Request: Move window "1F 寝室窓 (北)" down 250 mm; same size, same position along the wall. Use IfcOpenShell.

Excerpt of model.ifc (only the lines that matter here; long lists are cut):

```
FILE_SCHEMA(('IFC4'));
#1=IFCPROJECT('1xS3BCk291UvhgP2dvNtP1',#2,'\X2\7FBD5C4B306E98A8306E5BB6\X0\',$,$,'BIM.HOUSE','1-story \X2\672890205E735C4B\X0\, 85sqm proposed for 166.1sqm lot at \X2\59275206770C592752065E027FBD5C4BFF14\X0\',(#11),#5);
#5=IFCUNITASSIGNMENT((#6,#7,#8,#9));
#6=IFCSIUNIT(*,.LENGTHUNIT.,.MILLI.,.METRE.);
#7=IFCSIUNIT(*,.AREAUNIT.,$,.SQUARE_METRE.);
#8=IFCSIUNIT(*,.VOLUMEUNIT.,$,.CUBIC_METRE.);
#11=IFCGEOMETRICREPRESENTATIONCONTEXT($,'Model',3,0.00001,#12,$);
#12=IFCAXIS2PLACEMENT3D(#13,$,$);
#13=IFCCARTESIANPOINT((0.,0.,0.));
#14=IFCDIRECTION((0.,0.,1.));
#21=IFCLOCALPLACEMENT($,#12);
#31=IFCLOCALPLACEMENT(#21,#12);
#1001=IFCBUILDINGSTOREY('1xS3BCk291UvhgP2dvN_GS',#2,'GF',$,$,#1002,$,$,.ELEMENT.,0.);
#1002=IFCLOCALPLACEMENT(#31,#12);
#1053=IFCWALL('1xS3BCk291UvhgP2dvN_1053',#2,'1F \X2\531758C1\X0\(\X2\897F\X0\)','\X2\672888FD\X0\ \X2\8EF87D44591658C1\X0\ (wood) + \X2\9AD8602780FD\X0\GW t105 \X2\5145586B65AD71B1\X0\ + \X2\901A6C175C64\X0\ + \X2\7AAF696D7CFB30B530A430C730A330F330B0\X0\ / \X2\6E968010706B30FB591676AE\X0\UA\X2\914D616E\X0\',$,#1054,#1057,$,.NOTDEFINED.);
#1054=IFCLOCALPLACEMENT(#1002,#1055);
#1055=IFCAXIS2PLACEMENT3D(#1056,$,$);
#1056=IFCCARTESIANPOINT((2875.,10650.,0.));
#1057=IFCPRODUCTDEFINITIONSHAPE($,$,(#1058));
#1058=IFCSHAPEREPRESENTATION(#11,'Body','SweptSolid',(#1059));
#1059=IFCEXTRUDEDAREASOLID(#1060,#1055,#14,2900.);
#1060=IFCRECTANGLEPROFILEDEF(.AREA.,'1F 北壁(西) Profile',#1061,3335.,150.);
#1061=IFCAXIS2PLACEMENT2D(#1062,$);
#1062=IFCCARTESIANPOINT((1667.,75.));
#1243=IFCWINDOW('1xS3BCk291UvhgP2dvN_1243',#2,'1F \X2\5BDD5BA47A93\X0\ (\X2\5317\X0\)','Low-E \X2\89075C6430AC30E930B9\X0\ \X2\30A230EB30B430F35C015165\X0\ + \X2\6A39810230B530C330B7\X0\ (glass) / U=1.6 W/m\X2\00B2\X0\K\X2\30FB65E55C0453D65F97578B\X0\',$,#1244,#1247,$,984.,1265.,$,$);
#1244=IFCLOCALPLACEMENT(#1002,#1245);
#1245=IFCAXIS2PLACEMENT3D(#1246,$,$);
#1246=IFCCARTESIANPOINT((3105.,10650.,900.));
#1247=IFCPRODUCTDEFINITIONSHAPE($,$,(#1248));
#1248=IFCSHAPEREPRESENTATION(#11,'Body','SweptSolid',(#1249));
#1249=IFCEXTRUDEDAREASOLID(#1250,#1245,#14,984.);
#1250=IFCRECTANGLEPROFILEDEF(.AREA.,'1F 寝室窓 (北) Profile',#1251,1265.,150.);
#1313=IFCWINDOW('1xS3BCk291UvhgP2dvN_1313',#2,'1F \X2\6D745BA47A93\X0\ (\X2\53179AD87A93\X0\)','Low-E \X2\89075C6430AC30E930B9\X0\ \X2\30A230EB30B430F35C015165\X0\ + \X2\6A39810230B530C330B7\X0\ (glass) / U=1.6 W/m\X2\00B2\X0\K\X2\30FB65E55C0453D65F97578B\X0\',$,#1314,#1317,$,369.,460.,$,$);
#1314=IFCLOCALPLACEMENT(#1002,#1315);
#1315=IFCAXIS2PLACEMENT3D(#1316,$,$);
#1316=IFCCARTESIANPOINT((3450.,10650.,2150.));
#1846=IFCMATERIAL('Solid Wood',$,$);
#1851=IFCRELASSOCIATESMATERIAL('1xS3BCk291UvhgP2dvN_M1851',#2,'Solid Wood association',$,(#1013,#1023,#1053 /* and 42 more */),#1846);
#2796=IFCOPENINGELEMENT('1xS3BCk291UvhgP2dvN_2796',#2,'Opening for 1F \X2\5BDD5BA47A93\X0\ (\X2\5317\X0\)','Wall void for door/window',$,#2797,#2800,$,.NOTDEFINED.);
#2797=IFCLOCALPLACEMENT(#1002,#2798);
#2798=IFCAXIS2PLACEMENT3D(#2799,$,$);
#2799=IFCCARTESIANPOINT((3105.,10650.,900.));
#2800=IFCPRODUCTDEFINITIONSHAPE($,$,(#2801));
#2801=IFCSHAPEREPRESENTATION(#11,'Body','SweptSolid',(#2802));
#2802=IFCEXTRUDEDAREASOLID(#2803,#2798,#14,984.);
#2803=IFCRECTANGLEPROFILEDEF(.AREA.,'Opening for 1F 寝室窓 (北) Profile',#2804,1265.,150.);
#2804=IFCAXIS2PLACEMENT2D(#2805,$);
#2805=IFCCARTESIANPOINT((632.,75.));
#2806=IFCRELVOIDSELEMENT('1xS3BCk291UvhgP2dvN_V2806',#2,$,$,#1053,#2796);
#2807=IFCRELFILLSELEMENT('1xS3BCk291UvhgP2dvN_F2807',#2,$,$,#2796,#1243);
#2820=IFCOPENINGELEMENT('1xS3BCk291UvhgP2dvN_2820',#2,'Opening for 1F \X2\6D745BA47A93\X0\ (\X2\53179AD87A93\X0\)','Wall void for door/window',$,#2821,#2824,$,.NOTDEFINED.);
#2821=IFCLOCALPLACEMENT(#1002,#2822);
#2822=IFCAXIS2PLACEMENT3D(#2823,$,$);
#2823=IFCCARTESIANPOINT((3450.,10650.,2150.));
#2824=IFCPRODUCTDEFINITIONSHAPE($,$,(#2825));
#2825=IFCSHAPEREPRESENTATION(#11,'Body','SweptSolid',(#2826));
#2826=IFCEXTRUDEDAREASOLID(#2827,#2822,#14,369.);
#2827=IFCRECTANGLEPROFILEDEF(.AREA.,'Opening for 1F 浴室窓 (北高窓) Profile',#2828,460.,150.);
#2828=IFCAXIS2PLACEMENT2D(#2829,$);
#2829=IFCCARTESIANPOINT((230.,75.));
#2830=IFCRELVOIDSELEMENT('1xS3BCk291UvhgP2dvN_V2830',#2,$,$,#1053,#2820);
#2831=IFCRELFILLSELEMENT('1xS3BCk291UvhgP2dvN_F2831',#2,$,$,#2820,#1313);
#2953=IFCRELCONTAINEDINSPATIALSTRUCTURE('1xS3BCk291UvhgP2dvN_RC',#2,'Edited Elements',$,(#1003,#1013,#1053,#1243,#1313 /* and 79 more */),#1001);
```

```python
import numpy as np
import ifcopenshell
import ifcopenshell.api.geometry
import ifcopenshell.util.placement
import ifcopenshell.util.unit

model = ifcopenshell.open("model.ifc")
unit_scale = ifcopenshell.util.unit.calculate_unit_scale(model)

window = model.by_guid("1xS3BCk291UvhgP2dvN_1243")
opening = window.FillsVoids[0].RelatingOpeningElement
dz = -0.25 / unit_scale

shift = np.array([0.0, 0.0, dz])
# The window is not placed relative to its opening, so move both.
for product in (opening, window):
    matrix = ifcopenshell.util.placement.get_local_placement(product.ObjectPlacement)
    matrix[:3, 3] += shift
    ifcopenshell.api.geometry.edit_object_placement(model, product=product, matrix=matrix, is_si=False)

print(f"moved by {dz * unit_scale:+.3f} m")

model.write("model-out.ifc")
```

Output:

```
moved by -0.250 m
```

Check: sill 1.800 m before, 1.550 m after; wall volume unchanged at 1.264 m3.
